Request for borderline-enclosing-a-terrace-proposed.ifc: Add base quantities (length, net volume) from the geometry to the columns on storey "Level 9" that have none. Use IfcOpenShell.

First a look at what the model holds.

```python
import ifcopenshell
import ifcopenshell.util.element
import ifcopenshell.util.unit

model = ifcopenshell.open("borderline-enclosing-a-terrace-proposed.ifc")
print(model.schema)
for unit_type in ("LENGTHUNIT", "AREAUNIT", "VOLUMEUNIT"):
    print(unit_type, ifcopenshell.util.unit.calculate_unit_scale(model, unit_type))
storey = next(s for s in model.by_type("IfcBuildingStorey") if s.Name == "Level 9")
columns = [e for e in ifcopenshell.util.element.get_decomposition(storey) if e.is_a("IfcColumn")]
for e in sorted(columns, key=lambda e: e.id()):
    print(e.id(), e.is_a(), e.Name, list(ifcopenshell.util.element.get_psets(e, qtos_only=True)), sep=" | ")
```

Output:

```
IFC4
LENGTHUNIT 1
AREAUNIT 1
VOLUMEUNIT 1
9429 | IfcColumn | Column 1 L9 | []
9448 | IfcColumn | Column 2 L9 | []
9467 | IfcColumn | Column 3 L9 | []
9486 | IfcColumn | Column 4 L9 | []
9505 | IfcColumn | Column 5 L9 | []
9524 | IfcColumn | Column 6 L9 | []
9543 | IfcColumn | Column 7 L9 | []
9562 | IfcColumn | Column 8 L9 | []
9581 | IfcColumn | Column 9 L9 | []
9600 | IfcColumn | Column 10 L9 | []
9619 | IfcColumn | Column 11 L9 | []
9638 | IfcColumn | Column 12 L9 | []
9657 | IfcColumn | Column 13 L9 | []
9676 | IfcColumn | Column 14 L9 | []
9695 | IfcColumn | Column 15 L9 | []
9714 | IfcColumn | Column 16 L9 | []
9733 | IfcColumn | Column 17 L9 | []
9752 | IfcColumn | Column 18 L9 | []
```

```python
import ifcopenshell
import ifcopenshell.api.pset
import ifcopenshell.geom
import ifcopenshell.util.element
import ifcopenshell.util.shape
import ifcopenshell.util.unit

model = ifcopenshell.open("borderline-enclosing-a-terrace-proposed.ifc")
unit_scale = ifcopenshell.util.unit.calculate_unit_scale(model)
volume_scale = ifcopenshell.util.unit.calculate_unit_scale(model, "VOLUMEUNIT")
settings = ifcopenshell.geom.settings()

storey = next(s for s in model.by_type("IfcBuildingStorey") if s.Name == "Level 9")
columns = [e for e in ifcopenshell.util.element.get_decomposition(storey) if e.is_a("IfcColumn")]

for e in sorted(columns, key=lambda e: e.id()):
    if ifcopenshell.util.element.get_psets(e, qtos_only=True, should_inherit=False):
        continue
    # Geometry comes back in metres, in the element's own axes.
    shape = ifcopenshell.geom.create_shape(settings, e)
    values = {
        "Length": ifcopenshell.util.shape.get_z(shape.geometry) / unit_scale,
        "NetVolume": ifcopenshell.util.shape.get_volume(shape.geometry) / volume_scale,
    }
    qto = ifcopenshell.api.pset.add_qto(model, product=e, name="Qto_ColumnBaseQuantities")
    ifcopenshell.api.pset.edit_qto(model, qto=qto, properties=values)
    print(e.id(), {k: round(v, 3) for k, v in values.items()})

model.write("borderline-enclosing-a-terrace-proposed_v2.ifc")
```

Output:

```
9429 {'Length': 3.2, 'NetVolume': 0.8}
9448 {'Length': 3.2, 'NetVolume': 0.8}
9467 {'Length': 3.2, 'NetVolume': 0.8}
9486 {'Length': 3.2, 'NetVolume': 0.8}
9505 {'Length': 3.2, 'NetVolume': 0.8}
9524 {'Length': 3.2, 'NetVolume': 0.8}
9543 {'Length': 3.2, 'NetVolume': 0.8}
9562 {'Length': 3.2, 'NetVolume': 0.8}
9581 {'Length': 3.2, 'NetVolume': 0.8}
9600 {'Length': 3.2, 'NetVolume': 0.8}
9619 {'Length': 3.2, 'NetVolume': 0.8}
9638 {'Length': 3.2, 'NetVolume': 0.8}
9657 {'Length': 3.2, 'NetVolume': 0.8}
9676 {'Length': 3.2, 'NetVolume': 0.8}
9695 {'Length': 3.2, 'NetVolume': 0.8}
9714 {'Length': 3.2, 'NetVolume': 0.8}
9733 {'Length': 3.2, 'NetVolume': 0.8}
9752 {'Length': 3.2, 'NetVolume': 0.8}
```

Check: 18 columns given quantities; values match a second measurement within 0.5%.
